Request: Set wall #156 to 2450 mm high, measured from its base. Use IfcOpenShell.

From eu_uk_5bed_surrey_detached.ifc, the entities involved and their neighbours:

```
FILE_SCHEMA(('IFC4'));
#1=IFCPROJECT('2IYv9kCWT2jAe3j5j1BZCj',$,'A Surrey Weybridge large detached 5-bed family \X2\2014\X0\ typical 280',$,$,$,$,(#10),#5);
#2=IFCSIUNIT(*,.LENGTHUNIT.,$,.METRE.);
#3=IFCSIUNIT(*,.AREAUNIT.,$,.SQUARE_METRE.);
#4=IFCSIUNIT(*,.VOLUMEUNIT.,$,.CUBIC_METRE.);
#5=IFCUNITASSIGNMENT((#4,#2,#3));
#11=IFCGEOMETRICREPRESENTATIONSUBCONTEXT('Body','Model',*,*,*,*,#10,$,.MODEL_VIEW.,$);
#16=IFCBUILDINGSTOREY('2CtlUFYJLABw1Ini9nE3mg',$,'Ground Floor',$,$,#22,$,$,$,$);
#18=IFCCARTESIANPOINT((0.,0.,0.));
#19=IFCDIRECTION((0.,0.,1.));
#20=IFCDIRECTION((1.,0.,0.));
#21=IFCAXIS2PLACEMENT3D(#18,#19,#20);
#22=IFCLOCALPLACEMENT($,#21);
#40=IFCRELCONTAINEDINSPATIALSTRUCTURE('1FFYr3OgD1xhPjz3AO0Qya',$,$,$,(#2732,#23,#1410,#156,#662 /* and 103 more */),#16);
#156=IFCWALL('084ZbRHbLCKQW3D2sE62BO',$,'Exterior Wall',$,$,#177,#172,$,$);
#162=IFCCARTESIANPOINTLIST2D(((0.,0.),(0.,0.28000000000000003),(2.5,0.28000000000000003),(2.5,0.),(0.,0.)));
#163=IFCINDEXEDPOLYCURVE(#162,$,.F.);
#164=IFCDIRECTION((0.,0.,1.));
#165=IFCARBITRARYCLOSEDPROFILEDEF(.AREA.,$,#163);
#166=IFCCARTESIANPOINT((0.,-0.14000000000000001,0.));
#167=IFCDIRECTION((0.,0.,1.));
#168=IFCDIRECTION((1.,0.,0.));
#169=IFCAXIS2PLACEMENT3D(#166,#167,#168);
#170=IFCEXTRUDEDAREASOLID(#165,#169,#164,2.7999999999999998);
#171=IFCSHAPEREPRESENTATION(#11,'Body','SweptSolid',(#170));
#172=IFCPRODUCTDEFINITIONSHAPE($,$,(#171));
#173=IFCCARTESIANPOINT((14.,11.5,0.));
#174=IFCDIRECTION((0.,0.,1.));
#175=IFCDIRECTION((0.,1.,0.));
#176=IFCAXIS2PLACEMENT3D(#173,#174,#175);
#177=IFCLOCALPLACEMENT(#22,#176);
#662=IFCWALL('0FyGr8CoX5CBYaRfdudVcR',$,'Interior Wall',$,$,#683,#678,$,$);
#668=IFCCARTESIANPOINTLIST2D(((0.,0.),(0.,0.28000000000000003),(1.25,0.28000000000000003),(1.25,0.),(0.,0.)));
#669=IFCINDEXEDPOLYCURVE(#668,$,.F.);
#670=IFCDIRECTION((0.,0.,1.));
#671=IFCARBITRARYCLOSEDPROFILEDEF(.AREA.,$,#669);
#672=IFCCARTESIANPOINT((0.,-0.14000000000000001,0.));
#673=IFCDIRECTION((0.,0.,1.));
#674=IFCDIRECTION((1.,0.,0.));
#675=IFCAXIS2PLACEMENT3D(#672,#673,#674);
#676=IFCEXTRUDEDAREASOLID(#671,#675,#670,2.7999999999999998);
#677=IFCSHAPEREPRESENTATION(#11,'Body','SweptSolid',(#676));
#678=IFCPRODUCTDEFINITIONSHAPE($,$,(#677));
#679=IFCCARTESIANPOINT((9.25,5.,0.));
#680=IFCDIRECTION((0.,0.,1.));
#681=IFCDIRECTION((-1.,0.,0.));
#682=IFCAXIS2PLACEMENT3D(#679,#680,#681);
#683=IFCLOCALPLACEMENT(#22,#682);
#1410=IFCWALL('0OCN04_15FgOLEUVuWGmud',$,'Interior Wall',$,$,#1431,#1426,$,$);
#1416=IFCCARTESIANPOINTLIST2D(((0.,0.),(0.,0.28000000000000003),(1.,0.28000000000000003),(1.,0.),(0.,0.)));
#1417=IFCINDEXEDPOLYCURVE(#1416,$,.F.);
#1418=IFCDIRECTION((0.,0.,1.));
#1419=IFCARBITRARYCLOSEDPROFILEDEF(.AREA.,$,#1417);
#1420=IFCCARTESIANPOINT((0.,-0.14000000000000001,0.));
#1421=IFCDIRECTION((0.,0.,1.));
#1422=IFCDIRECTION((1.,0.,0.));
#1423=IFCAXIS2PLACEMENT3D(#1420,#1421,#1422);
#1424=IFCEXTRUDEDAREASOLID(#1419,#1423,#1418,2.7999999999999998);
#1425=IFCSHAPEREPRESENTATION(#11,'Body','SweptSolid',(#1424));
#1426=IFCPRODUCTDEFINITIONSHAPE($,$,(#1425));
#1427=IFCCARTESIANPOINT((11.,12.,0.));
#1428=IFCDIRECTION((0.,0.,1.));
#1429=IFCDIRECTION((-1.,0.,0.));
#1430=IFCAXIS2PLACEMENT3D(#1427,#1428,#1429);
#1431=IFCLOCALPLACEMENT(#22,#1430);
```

```python
import ifcopenshell
import ifcopenshell.geom
import ifcopenshell.util.representation
import ifcopenshell.util.shape
import ifcopenshell.util.unit

model = ifcopenshell.open("eu_uk_5bed_surrey_detached.ifc")
unit_scale = ifcopenshell.util.unit.calculate_unit_scale(model)
settings = ifcopenshell.geom.settings()


def volume(element):
    """Net volume in cubic metres, openings subtracted."""
    shape = ifcopenshell.geom.create_shape(settings, element)
    return ifcopenshell.util.shape.get_volume(shape.geometry)


wall = model.by_id(156)
before = volume(wall)

body = ifcopenshell.util.representation.get_representation(wall, "Model", "Body")
solid = body.Items[0]
old_height = solid.Depth
solid.Depth = 2.45 / unit_scale
after = volume(wall)

print(f"height {old_height:g} -> {solid.Depth:g}, volume {before:.3f} -> {after:.3f} m3")

model.write("eu_uk_5bed_surrey_detached_v2.ifc")
```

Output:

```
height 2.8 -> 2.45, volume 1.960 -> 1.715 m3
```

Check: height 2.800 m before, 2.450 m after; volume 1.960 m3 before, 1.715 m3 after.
